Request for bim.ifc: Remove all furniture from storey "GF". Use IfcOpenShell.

First a look at what the model holds.

```python
import ifcopenshell
import ifcopenshell.util.element

model = ifcopenshell.open("bim.ifc")
print(model.schema)
storey = next(s for s in model.by_type("IfcBuildingStorey") if s.Name == "GF")
furniture = [e for e in ifcopenshell.util.element.get_decomposition(storey) if e.is_a("IfcFurnishingElement")]
seen = {}
for e in furniture:
    element_type = ifcopenshell.util.element.get_type(e)
    name = element_type.Name if element_type not in (None, e) else None
    seen[name] = seen.get(name, 0) + 1
for name, count in sorted(seen.items(), key=str):
    print(count, "x", name)
```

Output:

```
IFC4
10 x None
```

```python
import ifcopenshell
import ifcopenshell.api.root
import ifcopenshell.util.element

model = ifcopenshell.open("bim.ifc")

storey = next(s for s in model.by_type("IfcBuildingStorey") if s.Name == "GF")
furniture = [e for e in ifcopenshell.util.element.get_decomposition(storey) if e.is_a("IfcFurnishingElement")]

for e in furniture:
    ifcopenshell.api.root.remove_product(model, product=e)
print(len(furniture), "removed")

model.write("bim-out.ifc")
```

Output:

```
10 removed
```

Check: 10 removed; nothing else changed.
